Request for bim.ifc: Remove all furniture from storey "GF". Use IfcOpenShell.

First a look at what the model holds.

```python
import ifcopenshell
import ifcopenshell.util.element

model = ifcopenshell.open("bim.ifc")
print(model.schema)
storey = next(s for s in model.by_type("IfcBuildingStorey") if s.Name == "GF")
furniture = [e for e in ifcopenshell.util.element.get_decomposition(storey) if e.is_a("IfcFurnishingElement")]
seen = {}
for e in furniture:
    element_type = ifcopenshell.util.element.get_type(e)
    name = element_type.Name if element_type not in (None, e) else None
    seen[name] = seen.get(name, 0) + 1
for name, count in sorted(seen.items(), key=str):
    print(count, "x", name)
```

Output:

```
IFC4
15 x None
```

```python
import ifcopenshell
import ifcopenshell.api.root
import ifcopenshell.util.element

model = ifcopenshell.open("bim.ifc")

storey = next(s for s in model.by_type("IfcBuildingStorey") if s.Name == "GF")
furniture = [e for e in ifcopenshell.util.element.get_decomposition(storey) if e.is_a("IfcFurnishingElement")]

for e in furniture:
    ifcopenshell.api.root.remove_product(model, product=e)
print(len(furniture), "removed")

model.write("bim_updated.ifc")
```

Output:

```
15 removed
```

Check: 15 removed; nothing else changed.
